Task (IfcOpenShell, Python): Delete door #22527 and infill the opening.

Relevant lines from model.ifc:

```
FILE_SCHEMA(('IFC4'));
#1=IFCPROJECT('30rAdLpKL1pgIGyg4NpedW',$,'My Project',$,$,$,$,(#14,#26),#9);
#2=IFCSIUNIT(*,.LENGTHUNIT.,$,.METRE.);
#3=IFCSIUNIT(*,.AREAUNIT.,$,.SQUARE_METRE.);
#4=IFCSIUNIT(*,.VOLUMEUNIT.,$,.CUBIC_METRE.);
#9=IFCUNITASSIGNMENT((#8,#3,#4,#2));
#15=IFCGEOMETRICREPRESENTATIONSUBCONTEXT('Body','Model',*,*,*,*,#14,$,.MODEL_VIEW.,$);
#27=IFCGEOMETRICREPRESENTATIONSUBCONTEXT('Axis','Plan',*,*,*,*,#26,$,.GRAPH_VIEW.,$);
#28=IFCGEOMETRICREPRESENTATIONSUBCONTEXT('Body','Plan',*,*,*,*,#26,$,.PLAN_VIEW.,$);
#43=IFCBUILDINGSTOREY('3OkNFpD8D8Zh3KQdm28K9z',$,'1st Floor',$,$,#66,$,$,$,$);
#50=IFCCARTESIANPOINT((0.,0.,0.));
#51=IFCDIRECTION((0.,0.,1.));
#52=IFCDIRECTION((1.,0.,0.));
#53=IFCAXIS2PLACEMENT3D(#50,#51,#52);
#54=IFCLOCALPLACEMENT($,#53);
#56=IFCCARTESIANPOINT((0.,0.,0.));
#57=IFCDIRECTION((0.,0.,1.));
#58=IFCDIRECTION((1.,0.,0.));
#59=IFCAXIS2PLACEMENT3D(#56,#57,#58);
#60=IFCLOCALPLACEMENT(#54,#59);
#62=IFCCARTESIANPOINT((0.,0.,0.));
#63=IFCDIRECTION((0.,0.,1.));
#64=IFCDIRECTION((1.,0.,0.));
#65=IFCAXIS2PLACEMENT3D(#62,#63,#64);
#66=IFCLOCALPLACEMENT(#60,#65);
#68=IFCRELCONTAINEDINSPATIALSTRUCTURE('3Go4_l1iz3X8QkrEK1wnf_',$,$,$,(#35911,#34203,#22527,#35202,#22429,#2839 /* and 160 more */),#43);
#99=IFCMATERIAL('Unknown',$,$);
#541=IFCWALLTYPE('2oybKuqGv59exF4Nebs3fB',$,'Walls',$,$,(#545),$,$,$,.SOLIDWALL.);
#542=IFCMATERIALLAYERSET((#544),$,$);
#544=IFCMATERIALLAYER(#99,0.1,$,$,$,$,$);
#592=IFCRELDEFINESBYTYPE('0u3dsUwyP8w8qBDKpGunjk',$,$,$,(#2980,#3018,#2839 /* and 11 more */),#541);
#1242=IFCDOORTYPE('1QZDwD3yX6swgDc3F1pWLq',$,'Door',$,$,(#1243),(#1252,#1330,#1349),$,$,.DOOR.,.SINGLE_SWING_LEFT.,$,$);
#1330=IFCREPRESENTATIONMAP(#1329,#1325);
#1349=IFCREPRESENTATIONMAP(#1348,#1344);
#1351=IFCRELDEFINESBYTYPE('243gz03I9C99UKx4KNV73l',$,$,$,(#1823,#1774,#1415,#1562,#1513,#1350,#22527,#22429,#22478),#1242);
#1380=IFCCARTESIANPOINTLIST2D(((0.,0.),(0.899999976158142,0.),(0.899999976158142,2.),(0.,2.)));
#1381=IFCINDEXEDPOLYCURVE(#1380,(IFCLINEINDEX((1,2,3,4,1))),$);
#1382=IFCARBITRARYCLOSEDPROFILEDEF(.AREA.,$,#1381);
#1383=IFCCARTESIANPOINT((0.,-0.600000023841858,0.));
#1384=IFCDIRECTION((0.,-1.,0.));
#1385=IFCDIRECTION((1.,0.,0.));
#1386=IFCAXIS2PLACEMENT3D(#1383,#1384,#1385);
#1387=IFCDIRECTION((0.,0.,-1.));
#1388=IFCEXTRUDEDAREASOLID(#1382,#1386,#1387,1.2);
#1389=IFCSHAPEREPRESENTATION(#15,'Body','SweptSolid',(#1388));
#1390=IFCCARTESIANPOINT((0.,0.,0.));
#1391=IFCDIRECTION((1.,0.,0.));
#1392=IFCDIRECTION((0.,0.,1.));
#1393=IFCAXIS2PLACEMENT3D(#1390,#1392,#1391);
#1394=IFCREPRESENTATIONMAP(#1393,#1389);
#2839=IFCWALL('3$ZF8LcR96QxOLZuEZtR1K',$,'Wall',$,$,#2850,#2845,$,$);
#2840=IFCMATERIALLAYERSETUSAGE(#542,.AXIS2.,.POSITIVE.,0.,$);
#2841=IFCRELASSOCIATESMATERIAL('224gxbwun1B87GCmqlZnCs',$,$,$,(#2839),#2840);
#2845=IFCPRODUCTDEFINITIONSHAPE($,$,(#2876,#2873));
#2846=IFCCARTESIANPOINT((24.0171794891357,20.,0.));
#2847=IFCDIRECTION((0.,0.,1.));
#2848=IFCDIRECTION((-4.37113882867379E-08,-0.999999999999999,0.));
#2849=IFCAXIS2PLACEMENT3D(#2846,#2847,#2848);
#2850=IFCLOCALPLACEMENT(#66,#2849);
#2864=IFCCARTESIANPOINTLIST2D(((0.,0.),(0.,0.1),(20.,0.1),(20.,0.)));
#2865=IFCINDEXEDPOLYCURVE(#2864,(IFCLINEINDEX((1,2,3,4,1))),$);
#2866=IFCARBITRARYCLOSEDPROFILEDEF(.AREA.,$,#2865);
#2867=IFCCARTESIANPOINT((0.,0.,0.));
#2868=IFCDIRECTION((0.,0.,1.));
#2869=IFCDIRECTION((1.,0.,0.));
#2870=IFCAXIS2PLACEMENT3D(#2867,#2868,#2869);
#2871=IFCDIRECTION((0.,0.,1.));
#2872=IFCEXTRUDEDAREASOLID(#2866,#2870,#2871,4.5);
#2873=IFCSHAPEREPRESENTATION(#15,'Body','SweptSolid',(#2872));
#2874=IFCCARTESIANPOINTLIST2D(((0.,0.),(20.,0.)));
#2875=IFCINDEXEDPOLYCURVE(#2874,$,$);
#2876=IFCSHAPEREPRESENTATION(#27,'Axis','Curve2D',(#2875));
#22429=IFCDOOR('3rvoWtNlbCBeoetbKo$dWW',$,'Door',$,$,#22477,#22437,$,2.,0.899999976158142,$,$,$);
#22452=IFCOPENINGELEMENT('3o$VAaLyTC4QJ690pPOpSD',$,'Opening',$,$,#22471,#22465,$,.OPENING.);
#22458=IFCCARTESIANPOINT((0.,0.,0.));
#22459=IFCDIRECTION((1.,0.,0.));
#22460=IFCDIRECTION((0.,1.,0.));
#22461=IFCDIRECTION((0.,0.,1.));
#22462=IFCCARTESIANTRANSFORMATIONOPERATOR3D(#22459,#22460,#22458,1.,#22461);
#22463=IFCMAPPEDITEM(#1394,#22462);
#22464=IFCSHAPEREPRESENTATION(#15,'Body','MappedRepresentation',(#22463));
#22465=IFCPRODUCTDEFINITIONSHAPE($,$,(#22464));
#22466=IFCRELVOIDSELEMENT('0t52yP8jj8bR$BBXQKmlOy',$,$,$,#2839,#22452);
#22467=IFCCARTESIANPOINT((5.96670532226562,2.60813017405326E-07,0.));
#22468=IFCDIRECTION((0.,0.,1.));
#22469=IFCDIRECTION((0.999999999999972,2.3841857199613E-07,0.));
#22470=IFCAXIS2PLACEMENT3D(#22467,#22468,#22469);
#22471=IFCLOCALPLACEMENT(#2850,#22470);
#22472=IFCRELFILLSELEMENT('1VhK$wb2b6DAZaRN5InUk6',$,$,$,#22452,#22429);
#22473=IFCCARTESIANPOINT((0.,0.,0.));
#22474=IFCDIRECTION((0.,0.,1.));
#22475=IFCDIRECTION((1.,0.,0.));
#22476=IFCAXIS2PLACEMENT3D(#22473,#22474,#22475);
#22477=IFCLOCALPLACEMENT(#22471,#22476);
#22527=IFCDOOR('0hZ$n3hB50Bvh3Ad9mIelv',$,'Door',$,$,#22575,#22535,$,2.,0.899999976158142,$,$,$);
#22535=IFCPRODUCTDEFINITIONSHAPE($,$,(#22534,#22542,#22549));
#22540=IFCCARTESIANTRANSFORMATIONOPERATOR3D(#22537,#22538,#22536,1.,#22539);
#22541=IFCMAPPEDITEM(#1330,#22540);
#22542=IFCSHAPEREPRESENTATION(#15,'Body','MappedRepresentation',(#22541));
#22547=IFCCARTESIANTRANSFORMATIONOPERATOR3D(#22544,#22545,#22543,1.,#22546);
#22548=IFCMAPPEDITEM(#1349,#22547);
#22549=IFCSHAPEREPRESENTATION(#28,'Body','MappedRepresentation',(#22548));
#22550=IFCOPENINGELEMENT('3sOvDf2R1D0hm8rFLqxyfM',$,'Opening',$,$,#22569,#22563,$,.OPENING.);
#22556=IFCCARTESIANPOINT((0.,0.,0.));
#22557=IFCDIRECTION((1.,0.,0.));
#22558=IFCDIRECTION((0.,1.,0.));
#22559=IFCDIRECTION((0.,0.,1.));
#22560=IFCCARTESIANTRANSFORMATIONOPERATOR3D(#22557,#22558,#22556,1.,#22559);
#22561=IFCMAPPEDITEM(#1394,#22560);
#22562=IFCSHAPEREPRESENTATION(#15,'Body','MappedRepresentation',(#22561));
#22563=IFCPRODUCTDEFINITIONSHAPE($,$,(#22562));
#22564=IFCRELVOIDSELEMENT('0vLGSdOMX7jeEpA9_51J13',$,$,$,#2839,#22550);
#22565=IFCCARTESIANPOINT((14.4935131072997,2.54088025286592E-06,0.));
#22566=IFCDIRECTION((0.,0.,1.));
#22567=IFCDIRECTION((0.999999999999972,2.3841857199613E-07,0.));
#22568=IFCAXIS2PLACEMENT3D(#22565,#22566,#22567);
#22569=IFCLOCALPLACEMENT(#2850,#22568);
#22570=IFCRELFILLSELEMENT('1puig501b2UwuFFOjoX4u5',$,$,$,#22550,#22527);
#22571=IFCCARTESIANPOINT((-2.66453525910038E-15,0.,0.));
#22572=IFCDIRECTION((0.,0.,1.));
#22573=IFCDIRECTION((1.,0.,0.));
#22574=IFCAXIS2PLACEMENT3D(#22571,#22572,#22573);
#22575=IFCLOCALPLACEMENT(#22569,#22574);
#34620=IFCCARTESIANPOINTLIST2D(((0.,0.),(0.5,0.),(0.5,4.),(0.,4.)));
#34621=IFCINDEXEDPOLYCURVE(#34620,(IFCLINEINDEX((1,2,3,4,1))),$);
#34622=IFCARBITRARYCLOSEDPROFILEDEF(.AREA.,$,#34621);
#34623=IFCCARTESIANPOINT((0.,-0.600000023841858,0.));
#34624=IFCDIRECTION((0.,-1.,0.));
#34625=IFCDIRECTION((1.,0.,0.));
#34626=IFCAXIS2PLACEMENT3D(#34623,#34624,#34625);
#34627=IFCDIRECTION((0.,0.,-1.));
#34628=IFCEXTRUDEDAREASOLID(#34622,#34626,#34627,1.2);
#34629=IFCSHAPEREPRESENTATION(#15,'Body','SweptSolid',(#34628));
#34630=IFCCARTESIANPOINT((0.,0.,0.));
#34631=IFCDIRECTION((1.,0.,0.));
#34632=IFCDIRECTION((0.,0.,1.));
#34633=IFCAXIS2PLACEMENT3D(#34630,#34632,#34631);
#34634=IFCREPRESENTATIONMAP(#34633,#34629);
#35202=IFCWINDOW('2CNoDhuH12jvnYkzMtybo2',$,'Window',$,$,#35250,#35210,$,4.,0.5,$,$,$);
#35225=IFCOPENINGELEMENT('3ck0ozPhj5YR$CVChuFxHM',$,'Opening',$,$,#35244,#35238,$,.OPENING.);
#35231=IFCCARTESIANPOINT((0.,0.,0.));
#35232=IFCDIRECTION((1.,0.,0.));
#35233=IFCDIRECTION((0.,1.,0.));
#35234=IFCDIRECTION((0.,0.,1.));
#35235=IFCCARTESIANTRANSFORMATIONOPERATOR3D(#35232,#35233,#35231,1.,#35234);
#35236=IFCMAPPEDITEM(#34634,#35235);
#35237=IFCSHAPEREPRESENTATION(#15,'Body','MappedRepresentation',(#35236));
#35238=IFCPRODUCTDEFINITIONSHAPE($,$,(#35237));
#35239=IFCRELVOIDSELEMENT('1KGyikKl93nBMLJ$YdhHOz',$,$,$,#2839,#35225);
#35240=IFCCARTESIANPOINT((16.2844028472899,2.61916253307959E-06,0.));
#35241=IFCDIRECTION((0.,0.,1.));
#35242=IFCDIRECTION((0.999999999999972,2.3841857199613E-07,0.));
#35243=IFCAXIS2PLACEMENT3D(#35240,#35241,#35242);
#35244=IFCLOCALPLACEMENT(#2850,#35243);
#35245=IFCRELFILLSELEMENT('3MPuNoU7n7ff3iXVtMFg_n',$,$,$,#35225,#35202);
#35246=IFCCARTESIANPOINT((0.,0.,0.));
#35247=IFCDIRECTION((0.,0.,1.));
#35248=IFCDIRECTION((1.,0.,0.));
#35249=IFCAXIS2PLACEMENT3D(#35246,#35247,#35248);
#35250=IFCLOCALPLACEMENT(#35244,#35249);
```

```python
import ifcopenshell
import ifcopenshell.api.feature
import ifcopenshell.api.root
import ifcopenshell.geom
import ifcopenshell.util.shape

model = ifcopenshell.open("model.ifc")
settings = ifcopenshell.geom.settings()


def volume(element):
    """Net volume in cubic metres, openings subtracted."""
    shape = ifcopenshell.geom.create_shape(settings, element)
    return ifcopenshell.util.shape.get_volume(shape.geometry)


door = model.by_guid("0hZ$n3hB50Bvh3Ad9mIelv")
opening = door.FillsVoids[0].RelatingOpeningElement
wall = opening.VoidsElements[0].RelatingBuildingElement
before = volume(wall)

ifcopenshell.api.root.remove_product(model, product=door)
ifcopenshell.api.feature.remove_feature(model, feature=opening)

after = volume(wall)

print(f"wall volume {before:.3f} -> {after:.3f} m3")

model.write("model_edited.ifc")
```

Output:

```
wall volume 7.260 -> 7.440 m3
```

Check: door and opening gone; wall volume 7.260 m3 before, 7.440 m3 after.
